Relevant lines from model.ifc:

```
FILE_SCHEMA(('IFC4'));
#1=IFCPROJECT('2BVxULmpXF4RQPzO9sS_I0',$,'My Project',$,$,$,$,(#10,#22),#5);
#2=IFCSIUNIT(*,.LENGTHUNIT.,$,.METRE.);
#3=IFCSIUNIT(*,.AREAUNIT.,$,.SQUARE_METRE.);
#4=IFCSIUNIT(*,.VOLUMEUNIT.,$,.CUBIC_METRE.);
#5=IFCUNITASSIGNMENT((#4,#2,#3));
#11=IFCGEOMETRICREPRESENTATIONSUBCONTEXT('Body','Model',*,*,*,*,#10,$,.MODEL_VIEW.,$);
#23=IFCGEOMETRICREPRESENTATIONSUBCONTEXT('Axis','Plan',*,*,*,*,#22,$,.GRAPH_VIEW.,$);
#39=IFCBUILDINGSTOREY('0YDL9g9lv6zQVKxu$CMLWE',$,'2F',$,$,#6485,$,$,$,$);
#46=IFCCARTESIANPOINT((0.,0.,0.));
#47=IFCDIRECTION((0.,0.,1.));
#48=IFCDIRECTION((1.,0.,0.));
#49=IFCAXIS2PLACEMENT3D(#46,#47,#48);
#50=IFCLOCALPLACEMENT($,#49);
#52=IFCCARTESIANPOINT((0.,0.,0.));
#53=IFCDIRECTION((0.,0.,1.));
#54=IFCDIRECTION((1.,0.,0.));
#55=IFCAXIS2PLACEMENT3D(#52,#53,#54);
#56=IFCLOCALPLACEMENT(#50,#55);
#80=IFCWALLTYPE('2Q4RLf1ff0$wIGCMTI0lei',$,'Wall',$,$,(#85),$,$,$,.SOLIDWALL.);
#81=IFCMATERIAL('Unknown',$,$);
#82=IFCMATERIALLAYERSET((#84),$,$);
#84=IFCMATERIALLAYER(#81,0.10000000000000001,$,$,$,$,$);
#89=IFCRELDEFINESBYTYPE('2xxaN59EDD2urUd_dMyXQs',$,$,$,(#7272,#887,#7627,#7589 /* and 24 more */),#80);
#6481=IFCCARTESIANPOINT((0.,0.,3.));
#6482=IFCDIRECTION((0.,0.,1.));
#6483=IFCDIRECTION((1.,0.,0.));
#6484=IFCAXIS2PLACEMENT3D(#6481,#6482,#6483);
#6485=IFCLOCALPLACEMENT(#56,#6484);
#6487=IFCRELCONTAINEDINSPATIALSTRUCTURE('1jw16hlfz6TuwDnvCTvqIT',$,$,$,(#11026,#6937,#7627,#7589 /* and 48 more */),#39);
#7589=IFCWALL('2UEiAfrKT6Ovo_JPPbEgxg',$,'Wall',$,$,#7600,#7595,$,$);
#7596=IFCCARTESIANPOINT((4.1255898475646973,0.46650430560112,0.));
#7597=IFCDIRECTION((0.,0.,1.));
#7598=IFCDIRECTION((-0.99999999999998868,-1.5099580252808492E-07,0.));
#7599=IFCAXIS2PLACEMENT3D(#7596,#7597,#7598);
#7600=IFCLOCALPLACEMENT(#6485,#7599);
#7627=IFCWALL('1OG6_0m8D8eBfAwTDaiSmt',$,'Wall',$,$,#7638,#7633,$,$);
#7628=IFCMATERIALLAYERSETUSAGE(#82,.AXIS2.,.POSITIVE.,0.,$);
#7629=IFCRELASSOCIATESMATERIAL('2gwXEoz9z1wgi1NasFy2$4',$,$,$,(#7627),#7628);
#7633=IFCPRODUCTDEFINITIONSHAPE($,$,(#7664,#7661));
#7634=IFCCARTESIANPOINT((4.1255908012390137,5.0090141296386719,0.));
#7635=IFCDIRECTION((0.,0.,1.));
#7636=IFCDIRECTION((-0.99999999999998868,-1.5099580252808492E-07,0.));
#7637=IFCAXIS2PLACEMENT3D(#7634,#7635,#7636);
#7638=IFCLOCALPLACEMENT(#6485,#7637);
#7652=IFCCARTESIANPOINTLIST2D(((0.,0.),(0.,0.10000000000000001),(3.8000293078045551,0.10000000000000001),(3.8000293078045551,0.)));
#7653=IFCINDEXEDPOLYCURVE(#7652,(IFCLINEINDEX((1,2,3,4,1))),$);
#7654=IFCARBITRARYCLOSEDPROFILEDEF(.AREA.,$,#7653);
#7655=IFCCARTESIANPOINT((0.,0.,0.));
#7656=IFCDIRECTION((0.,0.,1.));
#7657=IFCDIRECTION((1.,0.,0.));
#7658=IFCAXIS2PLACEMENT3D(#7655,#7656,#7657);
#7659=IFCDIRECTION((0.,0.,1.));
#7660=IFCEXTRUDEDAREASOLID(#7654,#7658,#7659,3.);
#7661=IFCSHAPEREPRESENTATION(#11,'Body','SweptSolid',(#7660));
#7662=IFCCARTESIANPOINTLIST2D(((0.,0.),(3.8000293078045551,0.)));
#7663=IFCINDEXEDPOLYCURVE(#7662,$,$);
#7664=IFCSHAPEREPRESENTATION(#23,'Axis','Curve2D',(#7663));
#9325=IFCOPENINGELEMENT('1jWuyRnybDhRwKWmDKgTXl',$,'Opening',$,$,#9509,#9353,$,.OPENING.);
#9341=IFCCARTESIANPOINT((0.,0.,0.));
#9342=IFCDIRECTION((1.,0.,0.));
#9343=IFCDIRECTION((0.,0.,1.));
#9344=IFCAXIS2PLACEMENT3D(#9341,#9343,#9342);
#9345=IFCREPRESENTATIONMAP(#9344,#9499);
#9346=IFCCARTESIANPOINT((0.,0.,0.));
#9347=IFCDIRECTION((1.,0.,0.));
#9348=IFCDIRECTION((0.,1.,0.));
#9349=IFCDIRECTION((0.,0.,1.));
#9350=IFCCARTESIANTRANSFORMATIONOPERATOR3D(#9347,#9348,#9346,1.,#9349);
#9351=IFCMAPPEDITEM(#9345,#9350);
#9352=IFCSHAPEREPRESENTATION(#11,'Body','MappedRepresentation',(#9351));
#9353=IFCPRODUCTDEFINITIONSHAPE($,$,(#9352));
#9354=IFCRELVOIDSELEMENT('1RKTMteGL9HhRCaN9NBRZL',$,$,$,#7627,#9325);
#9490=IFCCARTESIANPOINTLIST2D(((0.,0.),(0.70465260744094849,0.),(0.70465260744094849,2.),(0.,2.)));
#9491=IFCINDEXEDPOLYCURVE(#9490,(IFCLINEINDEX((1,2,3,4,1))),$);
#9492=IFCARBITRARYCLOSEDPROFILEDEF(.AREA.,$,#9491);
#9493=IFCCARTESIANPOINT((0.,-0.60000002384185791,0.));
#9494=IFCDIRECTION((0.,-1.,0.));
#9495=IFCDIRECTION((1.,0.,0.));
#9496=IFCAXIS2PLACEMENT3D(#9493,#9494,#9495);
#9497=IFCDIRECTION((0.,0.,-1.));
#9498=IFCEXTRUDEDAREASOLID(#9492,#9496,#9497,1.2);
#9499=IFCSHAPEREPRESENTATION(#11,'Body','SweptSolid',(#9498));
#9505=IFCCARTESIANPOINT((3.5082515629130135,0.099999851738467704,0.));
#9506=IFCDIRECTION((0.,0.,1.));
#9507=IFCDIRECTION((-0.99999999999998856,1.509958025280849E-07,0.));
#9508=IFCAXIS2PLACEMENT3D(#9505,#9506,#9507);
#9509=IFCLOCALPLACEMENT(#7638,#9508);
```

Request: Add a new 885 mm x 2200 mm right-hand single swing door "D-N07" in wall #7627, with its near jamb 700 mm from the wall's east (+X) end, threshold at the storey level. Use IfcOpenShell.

```python
import numpy as np
import ifcopenshell
import ifcopenshell.api.feature
import ifcopenshell.api.geometry
import ifcopenshell.api.root
import ifcopenshell.api.spatial
import ifcopenshell.geom
import ifcopenshell.util.element
import ifcopenshell.util.placement
import ifcopenshell.util.representation
import ifcopenshell.util.shape
import ifcopenshell.util.unit

model = ifcopenshell.open("model.ifc")
unit_scale = ifcopenshell.util.unit.calculate_unit_scale(model)
settings = ifcopenshell.geom.settings()


def volume(element):
    """Net volume in cubic metres, openings subtracted."""
    shape = ifcopenshell.geom.create_shape(settings, element)
    return ifcopenshell.util.shape.get_volume(shape.geometry)


wall = model.by_guid("1OG6_0m8D8eBfAwTDaiSmt")
storey = ifcopenshell.util.element.get_container(wall, ifc_class="IfcBuildingStorey")
context = ifcopenshell.util.representation.get_context(model, "Model", "Body", "MODEL_VIEW")
before = volume(wall)

width, height, from_end, sill = 0.885, 2.2, 0.7, 0.0  # metres

# The wall runs along its own X axis, and the end named is its -X end.
wall_shape = ifcopenshell.geom.create_shape(settings, wall)
x, y, z = ifcopenshell.util.shape.get_vertices(wall_shape.geometry).T
start = x.min() + from_end
face, thickness = float(y.min()), float(y.max() - y.min())
wall_matrix = ifcopenshell.util.placement.get_local_placement(wall.ObjectPlacement)
level = ifcopenshell.util.placement.get_local_placement(storey.ObjectPlacement)[2, 3]


def in_wall(x, y):
    """Placement at x, y metres in the wall's axes, at sill height."""
    matrix = wall_matrix.copy()
    matrix[:, 3] = wall_matrix @ np.array([x / unit_scale, y / unit_scale, 0.0, 1.0])
    matrix[2, 3] = level + sill / unit_scale
    return matrix


# Opening: a box that overshoots both wall faces by 50 mm.
opening = ifcopenshell.api.root.create_entity(model, ifc_class="IfcOpeningElement", predefined_type="OPENING")
box = ifcopenshell.api.geometry.add_wall_representation(
    model, context=context, length=width, height=height, thickness=thickness + 0.1
)
ifcopenshell.api.geometry.assign_representation(model, product=opening, representation=box)
ifcopenshell.api.geometry.edit_object_placement(model, product=opening, matrix=in_wall(start, face - 0.05), is_si=False)
ifcopenshell.api.feature.add_feature(model, feature=opening, element=wall)

door = ifcopenshell.api.root.create_entity(model, ifc_class="IfcDoor", name="D-N07", predefined_type="DOOR")
door.OverallWidth, door.OverallHeight = width / unit_scale, height / unit_scale
door.OperationType = "SINGLE_SWING_RIGHT"
body = ifcopenshell.api.geometry.add_door_representation(
    model,
    context=context,
    overall_width=door.OverallWidth,
    overall_height=door.OverallHeight,
    operation_type="SINGLE_SWING_RIGHT",
    lining_properties={"LiningDepth": thickness / unit_scale, "ThresholdDepth": thickness / unit_scale},
)
ifcopenshell.api.geometry.assign_representation(model, product=door, representation=body)
ifcopenshell.api.spatial.assign_container(model, products=[door], relating_structure=storey)
ifcopenshell.api.feature.add_filling(model, opening=opening, element=door)

# The lining spans the wall, so the door starts at the wall face.
ifcopenshell.api.geometry.edit_object_placement(model, product=door, matrix=in_wall(start, face), is_si=False)

after = volume(wall)

print(f"wall volume {before:.3f} -> {after:.3f} m3")

model.write("model_v2.ifc")
```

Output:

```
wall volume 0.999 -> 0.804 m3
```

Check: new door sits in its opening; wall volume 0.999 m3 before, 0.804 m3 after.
